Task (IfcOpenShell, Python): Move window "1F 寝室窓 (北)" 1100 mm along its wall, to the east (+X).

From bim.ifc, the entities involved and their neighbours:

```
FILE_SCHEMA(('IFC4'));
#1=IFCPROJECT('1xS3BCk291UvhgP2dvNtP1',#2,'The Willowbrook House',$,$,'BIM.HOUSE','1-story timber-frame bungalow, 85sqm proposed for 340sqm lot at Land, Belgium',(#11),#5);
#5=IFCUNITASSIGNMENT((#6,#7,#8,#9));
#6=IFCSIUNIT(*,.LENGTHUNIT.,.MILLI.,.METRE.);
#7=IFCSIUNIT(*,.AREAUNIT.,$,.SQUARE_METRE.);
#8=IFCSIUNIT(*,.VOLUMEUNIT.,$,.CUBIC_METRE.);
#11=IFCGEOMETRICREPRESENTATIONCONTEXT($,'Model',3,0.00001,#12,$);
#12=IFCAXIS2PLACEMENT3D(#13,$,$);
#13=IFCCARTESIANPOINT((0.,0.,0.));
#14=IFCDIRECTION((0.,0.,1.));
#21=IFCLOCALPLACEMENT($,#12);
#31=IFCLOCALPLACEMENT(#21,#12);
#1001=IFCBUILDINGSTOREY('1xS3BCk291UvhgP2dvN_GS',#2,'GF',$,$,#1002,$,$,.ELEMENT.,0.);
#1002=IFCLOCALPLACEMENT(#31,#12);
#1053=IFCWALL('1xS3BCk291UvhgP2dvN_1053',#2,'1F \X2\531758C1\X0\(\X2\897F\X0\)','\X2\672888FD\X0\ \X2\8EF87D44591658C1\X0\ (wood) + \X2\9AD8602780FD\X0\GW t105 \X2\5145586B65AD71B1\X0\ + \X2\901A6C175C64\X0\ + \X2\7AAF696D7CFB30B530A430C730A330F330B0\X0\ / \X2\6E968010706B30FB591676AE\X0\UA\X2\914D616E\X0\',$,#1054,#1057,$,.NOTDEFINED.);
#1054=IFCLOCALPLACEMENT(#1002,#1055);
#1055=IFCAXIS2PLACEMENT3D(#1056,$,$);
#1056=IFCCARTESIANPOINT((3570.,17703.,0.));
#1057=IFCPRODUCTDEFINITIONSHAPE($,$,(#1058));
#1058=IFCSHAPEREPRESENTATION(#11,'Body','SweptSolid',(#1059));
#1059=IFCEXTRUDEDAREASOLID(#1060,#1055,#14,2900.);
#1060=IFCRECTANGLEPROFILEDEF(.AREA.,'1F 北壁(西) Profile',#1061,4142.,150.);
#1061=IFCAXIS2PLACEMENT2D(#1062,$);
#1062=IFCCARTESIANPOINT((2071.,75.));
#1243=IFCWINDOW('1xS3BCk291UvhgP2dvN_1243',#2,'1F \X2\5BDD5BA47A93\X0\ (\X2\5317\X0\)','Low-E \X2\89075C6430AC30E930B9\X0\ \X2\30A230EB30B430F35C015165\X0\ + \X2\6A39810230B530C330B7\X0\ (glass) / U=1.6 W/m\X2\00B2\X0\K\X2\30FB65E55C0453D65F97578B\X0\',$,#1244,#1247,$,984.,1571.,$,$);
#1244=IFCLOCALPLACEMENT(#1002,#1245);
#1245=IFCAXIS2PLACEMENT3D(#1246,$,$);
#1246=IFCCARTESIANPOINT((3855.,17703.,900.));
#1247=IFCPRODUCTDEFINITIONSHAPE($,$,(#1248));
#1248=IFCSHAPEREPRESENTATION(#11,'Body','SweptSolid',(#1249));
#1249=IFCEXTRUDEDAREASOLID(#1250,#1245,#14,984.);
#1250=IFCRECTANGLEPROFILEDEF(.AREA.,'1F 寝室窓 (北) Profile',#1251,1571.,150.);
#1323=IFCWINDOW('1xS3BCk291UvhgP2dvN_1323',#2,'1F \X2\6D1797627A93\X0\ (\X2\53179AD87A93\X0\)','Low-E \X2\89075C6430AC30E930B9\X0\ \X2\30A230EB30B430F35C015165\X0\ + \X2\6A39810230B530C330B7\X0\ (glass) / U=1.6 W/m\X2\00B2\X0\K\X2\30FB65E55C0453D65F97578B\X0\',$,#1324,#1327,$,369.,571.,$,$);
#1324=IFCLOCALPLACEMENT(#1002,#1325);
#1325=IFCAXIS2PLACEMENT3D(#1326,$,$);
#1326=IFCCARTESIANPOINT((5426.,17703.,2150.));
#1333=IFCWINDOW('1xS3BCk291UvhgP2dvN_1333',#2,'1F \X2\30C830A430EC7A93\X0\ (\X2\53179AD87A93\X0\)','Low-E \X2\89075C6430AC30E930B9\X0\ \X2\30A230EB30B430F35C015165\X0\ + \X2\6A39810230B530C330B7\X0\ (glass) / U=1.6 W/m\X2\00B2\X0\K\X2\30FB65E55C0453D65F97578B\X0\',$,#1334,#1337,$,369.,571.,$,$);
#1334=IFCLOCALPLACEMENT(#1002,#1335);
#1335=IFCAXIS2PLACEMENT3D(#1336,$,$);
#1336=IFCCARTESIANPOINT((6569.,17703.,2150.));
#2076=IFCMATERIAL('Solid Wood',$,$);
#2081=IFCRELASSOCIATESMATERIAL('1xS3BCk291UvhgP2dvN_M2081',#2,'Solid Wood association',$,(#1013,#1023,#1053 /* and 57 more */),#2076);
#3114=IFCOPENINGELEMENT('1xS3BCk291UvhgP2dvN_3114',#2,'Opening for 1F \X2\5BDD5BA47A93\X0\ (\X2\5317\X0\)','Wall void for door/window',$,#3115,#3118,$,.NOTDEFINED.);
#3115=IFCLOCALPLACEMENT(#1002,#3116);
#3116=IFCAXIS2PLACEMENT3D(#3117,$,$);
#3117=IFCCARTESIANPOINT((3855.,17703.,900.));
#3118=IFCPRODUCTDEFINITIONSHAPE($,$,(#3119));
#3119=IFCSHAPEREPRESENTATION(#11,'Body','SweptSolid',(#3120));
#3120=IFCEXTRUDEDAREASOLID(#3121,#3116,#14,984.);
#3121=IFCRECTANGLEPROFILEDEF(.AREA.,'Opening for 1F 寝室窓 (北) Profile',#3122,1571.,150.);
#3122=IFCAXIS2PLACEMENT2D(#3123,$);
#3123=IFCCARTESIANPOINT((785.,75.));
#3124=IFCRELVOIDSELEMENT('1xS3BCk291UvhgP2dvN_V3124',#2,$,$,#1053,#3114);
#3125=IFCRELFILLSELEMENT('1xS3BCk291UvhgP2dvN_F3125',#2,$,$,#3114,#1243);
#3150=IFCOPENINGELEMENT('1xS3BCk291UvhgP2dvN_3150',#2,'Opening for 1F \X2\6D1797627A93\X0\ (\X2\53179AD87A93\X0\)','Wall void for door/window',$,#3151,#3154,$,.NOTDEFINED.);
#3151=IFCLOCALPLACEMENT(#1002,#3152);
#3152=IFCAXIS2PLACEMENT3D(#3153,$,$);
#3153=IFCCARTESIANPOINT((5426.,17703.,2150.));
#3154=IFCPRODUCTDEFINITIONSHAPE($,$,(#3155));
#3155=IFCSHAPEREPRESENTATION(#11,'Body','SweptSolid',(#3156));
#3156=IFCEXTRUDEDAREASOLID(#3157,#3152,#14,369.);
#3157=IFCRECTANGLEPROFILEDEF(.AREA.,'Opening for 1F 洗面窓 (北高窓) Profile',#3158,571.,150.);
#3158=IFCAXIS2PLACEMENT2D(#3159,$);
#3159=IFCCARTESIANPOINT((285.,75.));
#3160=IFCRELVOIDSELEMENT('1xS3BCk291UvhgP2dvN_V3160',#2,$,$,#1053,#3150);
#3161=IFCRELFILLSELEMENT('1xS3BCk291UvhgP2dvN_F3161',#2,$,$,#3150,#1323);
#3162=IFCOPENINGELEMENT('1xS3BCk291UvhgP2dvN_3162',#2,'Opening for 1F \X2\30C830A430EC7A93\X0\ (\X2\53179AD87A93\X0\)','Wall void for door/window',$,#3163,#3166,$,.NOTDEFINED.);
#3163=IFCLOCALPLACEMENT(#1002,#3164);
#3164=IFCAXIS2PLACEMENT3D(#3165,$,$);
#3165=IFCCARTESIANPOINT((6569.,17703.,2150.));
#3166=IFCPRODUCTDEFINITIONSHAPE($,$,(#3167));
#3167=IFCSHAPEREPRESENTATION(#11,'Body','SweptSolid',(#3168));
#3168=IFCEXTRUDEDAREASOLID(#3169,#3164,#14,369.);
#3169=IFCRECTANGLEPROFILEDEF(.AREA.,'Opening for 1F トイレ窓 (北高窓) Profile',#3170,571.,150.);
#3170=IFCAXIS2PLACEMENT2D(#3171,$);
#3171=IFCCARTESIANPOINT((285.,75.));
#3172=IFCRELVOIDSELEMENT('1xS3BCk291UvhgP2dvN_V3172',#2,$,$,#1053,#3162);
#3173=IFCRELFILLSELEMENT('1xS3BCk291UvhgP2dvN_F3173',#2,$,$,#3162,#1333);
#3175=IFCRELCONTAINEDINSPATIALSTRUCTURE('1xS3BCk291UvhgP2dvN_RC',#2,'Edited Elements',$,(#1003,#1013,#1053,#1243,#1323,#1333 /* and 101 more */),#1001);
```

```python
import ifcopenshell
import ifcopenshell.api.geometry
import ifcopenshell.util.placement
import ifcopenshell.util.unit

model = ifcopenshell.open("bim.ifc")
unit_scale = ifcopenshell.util.unit.calculate_unit_scale(model)

window = model.by_guid("1xS3BCk291UvhgP2dvN_1243")
opening = window.FillsVoids[0].RelatingOpeningElement
wall = opening.VoidsElements[0].RelatingBuildingElement

wall_matrix = ifcopenshell.util.placement.get_local_placement(wall.ObjectPlacement)
shift = wall_matrix[:3, 0] * 1.1 / unit_scale
before = ifcopenshell.util.placement.get_local_placement(window.ObjectPlacement)[:3, 3].copy()

# The window is not placed relative to its opening, so move both.
for product in (opening, window):
    matrix = ifcopenshell.util.placement.get_local_placement(product.ObjectPlacement)
    matrix[:3, 3] += shift
    ifcopenshell.api.geometry.edit_object_placement(model, product=product, matrix=matrix, is_si=False)

after = ifcopenshell.util.placement.get_local_placement(window.ObjectPlacement)[:3, 3]
print("window moved by", (after - before).round(3) + 0.0)

model.write("bim_updated.ifc")
```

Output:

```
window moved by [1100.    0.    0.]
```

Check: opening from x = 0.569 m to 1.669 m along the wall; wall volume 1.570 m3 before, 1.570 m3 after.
